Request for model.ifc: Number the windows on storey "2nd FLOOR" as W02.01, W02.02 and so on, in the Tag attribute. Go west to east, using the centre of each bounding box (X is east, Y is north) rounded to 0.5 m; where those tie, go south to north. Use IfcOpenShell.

First a look at what the model holds.

```python
import ifcopenshell
import ifcopenshell.util.element
import ifcopenshell.util.placement

model = ifcopenshell.open("model.ifc")
print(model.schema)
storey = next(s for s in model.by_type("IfcBuildingStorey") if s.Name == "2nd FLOOR")
windows = [e for e in ifcopenshell.util.element.get_decomposition(storey) if e.is_a("IfcWindow")]
for e in sorted(windows, key=lambda e: e.id()):
    origin = ifcopenshell.util.placement.get_local_placement(e.ObjectPlacement)[:3, 3]
    print(e.id(), e.Tag, e.Name, origin.round(2) + 0.0, sep=" | ")
```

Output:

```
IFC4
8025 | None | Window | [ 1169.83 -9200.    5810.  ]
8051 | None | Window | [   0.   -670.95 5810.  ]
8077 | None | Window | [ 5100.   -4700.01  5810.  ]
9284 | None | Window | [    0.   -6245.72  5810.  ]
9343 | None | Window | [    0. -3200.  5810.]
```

```python
import ifcopenshell
import ifcopenshell.geom
import ifcopenshell.util.element
import ifcopenshell.util.shape

model = ifcopenshell.open("model.ifc")
settings = ifcopenshell.geom.settings()
settings.set("use-world-coords", True)


def centre(element):
    shape = ifcopenshell.geom.create_shape(settings, element)
    return ifcopenshell.util.shape.get_bbox_centroid(shape.geometry)


storey = next(s for s in model.by_type("IfcBuildingStorey") if s.Name == "2nd FLOOR")
windows = [e for e in ifcopenshell.util.element.get_decomposition(storey) if e.is_a("IfcWindow")]

# Insertion points can sit at a corner or the storey origin, so sort by the geometry (in metres).
centres = {e: centre(e) for e in windows}
windows.sort(key=lambda e: (round(centres[e][0] / 0.5), centres[e][1]))

for i, e in enumerate(windows, start=1):
    number = f"W02.{i:02d}"
    e.Tag = number
    print(e.id(), number)

model.write("model_edited.ifc")
```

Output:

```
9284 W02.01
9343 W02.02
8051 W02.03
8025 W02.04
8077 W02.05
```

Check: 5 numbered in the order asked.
